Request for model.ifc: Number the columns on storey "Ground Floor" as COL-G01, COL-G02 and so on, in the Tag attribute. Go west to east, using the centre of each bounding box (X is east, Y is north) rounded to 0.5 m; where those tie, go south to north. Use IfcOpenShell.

First a look at what the model holds.

```python
import ifcopenshell
import ifcopenshell.util.element
import ifcopenshell.util.placement

model = ifcopenshell.open("model.ifc")
print(model.schema)
storey = next(s for s in model.by_type("IfcBuildingStorey") if s.Name == "Ground Floor")
columns = [e for e in ifcopenshell.util.element.get_decomposition(storey) if e.is_a("IfcColumn")]
for e in sorted(columns, key=lambda e: e.id()):
    origin = ifcopenshell.util.placement.get_local_placement(e.ObjectPlacement)[:3, 3]
    print(e.id(), e.Tag, e.Name, origin.round(2) + 0.0, sep=" | ")
```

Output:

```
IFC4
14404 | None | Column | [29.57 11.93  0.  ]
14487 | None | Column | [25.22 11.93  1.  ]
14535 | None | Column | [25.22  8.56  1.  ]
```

```python
import ifcopenshell
import ifcopenshell.geom
import ifcopenshell.util.element
import ifcopenshell.util.shape

model = ifcopenshell.open("model.ifc")
settings = ifcopenshell.geom.settings()
settings.set("use-world-coords", True)


def centre(element):
    shape = ifcopenshell.geom.create_shape(settings, element)
    return ifcopenshell.util.shape.get_bbox_centroid(shape.geometry)


storey = next(s for s in model.by_type("IfcBuildingStorey") if s.Name == "Ground Floor")
columns = [e for e in ifcopenshell.util.element.get_decomposition(storey) if e.is_a("IfcColumn")]

# Insertion points can sit at a corner or the storey origin, so sort by the geometry (in metres).
centres = {e: centre(e) for e in columns}
columns.sort(key=lambda e: (round(centres[e][0] / 0.5), centres[e][1]))

for i, e in enumerate(columns, start=1):
    number = f"COL-G{i:02d}"
    e.Tag = number
    print(e.id(), number)

model.write("model_edited.ifc")
```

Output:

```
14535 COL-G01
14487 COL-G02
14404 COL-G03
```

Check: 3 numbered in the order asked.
